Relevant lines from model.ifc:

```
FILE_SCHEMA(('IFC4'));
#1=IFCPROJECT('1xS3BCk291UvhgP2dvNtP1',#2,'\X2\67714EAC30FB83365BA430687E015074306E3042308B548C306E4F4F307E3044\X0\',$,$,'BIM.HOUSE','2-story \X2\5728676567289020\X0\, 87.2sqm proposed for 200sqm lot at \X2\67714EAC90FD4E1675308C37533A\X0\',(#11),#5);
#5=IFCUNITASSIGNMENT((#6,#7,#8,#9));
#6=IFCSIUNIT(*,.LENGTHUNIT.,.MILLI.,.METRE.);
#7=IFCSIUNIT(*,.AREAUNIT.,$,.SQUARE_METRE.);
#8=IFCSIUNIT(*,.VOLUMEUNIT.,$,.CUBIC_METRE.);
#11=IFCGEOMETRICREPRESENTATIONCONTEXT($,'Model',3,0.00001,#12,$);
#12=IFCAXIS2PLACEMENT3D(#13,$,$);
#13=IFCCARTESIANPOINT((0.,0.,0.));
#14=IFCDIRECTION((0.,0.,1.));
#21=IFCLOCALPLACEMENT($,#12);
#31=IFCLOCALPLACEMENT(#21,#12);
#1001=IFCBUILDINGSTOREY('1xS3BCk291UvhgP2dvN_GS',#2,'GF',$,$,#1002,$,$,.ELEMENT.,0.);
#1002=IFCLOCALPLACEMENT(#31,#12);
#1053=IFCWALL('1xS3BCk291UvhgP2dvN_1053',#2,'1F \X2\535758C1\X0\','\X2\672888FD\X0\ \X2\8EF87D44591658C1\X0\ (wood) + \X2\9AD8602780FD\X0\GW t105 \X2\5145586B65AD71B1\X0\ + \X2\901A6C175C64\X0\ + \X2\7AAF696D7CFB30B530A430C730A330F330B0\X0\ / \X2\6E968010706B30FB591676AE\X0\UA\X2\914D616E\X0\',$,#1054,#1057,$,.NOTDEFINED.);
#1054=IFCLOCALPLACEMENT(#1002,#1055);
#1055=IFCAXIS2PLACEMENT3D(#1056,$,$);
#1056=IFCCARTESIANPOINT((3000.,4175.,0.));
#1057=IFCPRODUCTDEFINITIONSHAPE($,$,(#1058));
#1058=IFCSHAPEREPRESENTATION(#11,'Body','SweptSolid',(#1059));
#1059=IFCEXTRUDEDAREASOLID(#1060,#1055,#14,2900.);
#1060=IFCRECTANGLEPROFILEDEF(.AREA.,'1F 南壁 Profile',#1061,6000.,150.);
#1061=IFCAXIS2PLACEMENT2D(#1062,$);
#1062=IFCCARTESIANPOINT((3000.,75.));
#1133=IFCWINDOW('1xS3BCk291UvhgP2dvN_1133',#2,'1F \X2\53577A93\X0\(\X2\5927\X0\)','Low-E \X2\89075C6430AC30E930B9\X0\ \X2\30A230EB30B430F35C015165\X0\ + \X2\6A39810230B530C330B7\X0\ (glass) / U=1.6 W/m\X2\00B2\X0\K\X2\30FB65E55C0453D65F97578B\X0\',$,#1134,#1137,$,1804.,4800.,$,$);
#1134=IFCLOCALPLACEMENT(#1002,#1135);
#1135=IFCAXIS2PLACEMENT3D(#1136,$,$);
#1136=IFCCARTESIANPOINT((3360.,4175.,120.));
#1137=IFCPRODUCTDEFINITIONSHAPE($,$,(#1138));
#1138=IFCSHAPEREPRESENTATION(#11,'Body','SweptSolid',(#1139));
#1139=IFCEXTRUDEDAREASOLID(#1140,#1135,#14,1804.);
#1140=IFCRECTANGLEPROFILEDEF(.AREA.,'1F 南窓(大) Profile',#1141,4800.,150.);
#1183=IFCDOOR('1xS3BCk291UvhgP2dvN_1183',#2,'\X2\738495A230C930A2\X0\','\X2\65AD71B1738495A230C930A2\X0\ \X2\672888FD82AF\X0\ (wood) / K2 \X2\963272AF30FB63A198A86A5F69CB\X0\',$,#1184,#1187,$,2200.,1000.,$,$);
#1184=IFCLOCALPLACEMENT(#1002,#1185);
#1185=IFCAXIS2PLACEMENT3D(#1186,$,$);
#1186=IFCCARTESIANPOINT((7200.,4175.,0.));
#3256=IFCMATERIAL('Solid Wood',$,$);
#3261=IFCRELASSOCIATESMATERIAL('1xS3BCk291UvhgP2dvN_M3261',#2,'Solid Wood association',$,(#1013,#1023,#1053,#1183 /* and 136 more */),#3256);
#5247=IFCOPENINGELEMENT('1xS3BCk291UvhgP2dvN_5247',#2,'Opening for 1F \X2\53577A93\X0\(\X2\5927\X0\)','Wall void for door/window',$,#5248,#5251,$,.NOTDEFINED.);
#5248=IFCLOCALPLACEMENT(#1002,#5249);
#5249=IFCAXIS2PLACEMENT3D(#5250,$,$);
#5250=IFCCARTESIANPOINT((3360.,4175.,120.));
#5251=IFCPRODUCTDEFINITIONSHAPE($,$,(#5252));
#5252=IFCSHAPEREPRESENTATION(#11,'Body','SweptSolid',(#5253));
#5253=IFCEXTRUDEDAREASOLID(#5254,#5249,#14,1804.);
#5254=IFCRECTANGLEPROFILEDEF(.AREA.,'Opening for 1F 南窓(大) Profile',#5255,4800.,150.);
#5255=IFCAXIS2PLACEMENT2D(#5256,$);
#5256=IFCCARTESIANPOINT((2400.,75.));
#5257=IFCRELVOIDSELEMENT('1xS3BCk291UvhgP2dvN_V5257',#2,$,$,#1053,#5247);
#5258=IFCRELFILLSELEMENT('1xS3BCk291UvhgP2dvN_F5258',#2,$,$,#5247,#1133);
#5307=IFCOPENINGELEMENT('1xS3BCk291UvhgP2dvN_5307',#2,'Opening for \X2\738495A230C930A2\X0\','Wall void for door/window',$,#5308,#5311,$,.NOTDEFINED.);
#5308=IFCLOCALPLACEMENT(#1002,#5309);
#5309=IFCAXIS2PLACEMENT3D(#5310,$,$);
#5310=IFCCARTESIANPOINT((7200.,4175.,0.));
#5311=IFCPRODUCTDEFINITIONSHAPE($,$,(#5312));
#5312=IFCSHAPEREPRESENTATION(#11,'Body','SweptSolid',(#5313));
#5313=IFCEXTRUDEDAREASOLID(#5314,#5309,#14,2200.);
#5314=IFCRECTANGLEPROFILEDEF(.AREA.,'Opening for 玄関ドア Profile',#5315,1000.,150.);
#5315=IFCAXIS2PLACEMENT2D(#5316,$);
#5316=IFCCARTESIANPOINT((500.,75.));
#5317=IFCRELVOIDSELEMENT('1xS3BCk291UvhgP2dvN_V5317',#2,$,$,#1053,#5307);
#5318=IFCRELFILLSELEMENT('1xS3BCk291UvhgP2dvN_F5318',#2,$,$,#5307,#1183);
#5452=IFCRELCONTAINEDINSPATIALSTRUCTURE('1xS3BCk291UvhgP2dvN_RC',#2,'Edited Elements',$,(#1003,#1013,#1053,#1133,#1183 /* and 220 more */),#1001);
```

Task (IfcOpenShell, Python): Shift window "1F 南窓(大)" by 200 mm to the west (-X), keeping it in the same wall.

```python
import ifcopenshell
import ifcopenshell.api.geometry
import ifcopenshell.util.placement
import ifcopenshell.util.unit

model = ifcopenshell.open("model.ifc")
unit_scale = ifcopenshell.util.unit.calculate_unit_scale(model)

window = model.by_guid("1xS3BCk291UvhgP2dvN_1133")
opening = window.FillsVoids[0].RelatingOpeningElement
wall = opening.VoidsElements[0].RelatingBuildingElement

wall_matrix = ifcopenshell.util.placement.get_local_placement(wall.ObjectPlacement)
shift = wall_matrix[:3, 0] * -0.2 / unit_scale
before = ifcopenshell.util.placement.get_local_placement(window.ObjectPlacement)[:3, 3].copy()

# The window is not placed relative to its opening, so move both.
for product in (opening, window):
    matrix = ifcopenshell.util.placement.get_local_placement(product.ObjectPlacement)
    matrix[:3, 3] += shift
    ifcopenshell.api.geometry.edit_object_placement(model, product=product, matrix=matrix, is_si=False)

after = ifcopenshell.util.placement.get_local_placement(window.ObjectPlacement)[:3, 3]
print("window moved by", (after - before).round(3) + 0.0)

model.write("model_v2.ifc")
```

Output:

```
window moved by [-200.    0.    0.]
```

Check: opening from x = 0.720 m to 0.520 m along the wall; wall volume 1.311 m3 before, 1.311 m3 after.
